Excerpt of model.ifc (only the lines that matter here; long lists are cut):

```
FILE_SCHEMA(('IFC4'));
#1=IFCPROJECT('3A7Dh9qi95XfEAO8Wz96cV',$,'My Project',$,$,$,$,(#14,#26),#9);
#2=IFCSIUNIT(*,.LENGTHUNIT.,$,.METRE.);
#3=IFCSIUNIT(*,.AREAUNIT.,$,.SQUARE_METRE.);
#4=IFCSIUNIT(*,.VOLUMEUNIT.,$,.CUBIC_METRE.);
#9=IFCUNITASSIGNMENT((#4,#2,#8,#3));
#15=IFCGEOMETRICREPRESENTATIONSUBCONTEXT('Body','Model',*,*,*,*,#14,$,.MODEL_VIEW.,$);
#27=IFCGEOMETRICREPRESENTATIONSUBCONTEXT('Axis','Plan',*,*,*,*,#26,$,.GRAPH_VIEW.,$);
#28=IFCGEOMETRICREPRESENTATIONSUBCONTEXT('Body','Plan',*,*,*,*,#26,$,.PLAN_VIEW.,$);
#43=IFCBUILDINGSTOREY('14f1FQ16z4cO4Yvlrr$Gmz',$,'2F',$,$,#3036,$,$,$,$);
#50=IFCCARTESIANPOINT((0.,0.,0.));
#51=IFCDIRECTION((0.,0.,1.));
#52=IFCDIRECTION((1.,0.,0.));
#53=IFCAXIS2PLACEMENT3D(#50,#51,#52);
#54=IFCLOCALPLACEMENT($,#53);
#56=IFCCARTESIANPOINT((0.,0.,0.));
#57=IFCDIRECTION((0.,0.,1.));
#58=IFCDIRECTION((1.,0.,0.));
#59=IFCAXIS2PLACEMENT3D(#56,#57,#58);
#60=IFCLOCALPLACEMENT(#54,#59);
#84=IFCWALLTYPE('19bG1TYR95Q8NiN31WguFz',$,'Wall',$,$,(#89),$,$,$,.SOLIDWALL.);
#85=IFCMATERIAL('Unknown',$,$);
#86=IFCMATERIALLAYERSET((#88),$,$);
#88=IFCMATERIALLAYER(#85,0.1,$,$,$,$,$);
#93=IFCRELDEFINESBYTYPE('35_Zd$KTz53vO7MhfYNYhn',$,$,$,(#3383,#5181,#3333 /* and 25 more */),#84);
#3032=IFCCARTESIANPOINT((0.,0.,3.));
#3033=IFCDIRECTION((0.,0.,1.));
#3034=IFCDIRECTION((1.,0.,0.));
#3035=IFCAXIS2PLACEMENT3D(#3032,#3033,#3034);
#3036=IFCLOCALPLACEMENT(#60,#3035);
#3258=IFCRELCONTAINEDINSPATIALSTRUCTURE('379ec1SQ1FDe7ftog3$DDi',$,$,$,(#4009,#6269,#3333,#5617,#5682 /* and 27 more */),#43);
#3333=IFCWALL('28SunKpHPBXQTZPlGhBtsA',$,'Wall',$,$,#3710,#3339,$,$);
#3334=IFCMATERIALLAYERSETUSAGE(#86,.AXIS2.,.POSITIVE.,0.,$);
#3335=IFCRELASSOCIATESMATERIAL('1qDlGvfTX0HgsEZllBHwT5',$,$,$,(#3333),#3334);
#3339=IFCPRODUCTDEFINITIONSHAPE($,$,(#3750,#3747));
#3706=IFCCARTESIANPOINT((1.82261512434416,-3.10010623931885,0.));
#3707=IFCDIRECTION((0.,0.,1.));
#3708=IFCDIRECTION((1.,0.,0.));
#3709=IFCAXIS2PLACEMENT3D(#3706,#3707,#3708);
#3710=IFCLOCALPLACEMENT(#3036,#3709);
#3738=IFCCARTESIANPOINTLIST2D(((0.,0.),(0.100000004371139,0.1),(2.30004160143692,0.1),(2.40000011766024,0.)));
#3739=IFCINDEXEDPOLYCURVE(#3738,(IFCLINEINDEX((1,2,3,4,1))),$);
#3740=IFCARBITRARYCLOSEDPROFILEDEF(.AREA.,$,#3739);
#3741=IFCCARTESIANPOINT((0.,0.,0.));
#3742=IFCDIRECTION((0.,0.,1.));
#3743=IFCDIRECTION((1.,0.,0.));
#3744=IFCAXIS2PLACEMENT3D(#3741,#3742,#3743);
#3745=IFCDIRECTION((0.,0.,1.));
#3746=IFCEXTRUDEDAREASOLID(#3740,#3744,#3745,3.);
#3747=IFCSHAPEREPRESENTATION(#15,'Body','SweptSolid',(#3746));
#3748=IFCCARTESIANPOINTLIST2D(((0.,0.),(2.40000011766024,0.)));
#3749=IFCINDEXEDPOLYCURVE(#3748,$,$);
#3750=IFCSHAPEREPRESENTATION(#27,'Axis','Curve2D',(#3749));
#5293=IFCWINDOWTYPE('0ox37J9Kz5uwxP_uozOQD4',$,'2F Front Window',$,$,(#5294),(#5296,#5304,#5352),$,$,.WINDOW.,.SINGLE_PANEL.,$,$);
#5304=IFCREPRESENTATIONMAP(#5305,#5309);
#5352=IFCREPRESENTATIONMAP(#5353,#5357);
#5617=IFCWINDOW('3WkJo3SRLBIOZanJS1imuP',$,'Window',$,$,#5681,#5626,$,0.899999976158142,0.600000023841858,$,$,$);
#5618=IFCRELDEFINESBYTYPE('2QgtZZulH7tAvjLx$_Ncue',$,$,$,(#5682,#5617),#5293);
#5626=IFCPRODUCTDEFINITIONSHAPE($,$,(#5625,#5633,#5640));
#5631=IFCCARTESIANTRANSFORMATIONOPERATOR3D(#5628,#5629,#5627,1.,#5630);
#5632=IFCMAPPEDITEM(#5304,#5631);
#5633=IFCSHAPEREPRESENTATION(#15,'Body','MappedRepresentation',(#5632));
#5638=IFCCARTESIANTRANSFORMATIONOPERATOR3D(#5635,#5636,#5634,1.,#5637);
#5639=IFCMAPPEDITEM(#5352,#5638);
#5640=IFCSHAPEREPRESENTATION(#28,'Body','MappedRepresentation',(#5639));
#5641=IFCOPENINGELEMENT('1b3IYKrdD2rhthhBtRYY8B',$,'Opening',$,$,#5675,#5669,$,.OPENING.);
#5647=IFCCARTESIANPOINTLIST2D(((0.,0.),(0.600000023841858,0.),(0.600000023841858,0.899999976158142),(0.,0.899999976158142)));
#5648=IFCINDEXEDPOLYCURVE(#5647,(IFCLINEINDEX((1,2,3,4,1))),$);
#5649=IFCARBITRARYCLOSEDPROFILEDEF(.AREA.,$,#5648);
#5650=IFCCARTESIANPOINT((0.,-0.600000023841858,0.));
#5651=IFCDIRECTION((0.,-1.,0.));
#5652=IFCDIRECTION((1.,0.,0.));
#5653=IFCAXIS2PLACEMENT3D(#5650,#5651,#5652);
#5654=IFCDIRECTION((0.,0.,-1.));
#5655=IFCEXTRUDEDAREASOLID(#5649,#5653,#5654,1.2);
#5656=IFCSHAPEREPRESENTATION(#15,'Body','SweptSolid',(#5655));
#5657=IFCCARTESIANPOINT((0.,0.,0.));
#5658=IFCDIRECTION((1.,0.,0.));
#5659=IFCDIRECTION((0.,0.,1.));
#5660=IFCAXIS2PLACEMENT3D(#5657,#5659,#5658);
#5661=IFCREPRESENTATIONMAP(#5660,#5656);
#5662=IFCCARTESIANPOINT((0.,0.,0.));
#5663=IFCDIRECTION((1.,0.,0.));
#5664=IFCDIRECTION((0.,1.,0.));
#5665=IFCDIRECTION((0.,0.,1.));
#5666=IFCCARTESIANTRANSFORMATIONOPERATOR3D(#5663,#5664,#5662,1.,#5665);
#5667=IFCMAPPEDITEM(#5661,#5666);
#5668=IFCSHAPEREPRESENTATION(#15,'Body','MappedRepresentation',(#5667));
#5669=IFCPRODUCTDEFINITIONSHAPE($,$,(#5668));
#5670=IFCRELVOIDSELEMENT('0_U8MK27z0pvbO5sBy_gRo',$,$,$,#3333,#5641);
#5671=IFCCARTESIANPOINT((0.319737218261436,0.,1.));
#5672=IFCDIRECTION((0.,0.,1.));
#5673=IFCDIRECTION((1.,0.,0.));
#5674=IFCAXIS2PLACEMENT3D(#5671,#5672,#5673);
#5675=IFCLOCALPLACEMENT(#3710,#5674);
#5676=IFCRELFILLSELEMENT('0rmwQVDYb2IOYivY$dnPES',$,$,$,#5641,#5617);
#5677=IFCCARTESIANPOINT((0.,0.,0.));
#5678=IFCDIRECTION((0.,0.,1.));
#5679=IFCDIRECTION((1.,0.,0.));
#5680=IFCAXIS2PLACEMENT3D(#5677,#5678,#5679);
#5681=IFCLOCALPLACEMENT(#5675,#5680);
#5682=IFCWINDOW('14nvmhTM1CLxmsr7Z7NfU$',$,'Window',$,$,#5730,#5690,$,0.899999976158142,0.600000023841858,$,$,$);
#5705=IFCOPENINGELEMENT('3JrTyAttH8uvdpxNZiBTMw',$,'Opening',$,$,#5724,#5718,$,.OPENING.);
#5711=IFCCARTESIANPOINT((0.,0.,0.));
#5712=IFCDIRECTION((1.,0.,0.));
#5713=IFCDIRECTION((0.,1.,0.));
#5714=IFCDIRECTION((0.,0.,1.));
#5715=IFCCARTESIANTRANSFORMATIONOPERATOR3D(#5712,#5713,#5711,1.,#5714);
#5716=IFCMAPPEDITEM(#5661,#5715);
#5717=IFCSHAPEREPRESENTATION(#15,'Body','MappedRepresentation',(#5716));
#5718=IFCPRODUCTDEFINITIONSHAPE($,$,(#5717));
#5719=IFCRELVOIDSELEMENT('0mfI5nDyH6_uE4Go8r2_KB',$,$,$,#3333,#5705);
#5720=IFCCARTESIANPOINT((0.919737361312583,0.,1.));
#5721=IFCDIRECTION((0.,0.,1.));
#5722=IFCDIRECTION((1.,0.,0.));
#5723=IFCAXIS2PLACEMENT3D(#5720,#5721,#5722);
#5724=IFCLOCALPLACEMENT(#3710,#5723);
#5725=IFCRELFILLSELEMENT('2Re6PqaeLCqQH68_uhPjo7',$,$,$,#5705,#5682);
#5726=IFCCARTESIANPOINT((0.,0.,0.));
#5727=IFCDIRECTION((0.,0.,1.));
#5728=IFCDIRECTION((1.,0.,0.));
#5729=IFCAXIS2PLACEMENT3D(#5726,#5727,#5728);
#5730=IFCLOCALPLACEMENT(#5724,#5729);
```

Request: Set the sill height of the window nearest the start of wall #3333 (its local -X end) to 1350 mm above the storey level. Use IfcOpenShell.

```python
import numpy as np
import ifcopenshell
import ifcopenshell.api.geometry
import ifcopenshell.geom
import ifcopenshell.util.element
import ifcopenshell.util.placement
import ifcopenshell.util.shape
import ifcopenshell.util.unit

model = ifcopenshell.open("model.ifc")
unit_scale = ifcopenshell.util.unit.calculate_unit_scale(model)

window = model.by_id(5617)
opening = window.FillsVoids[0].RelatingOpeningElement
storey = ifcopenshell.util.element.get_container(window, ifc_class="IfcBuildingStorey")
level = ifcopenshell.util.placement.get_local_placement(storey.ObjectPlacement)[2, 3]

# The opening's origin need not be at the sill, so measure its lowest point.
shape = ifcopenshell.geom.create_shape(ifcopenshell.geom.settings(), opening)
bottom = ifcopenshell.util.shape.get_shape_bottom_elevation(shape, shape.geometry) / unit_scale
dz = level + 1.35 / unit_scale - bottom

shift = np.array([0.0, 0.0, dz])
# The window is placed relative to its opening, so it follows when the opening moves.
matrix = ifcopenshell.util.placement.get_local_placement(opening.ObjectPlacement)
matrix[:3, 3] += shift
ifcopenshell.api.geometry.edit_object_placement(
    model, product=opening, matrix=matrix, is_si=False, should_transform_children=True
)

print(f"moved by {dz * unit_scale:+.3f} m")

model.write("model_updated.ifc")
```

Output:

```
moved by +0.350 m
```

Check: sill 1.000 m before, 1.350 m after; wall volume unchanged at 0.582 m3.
